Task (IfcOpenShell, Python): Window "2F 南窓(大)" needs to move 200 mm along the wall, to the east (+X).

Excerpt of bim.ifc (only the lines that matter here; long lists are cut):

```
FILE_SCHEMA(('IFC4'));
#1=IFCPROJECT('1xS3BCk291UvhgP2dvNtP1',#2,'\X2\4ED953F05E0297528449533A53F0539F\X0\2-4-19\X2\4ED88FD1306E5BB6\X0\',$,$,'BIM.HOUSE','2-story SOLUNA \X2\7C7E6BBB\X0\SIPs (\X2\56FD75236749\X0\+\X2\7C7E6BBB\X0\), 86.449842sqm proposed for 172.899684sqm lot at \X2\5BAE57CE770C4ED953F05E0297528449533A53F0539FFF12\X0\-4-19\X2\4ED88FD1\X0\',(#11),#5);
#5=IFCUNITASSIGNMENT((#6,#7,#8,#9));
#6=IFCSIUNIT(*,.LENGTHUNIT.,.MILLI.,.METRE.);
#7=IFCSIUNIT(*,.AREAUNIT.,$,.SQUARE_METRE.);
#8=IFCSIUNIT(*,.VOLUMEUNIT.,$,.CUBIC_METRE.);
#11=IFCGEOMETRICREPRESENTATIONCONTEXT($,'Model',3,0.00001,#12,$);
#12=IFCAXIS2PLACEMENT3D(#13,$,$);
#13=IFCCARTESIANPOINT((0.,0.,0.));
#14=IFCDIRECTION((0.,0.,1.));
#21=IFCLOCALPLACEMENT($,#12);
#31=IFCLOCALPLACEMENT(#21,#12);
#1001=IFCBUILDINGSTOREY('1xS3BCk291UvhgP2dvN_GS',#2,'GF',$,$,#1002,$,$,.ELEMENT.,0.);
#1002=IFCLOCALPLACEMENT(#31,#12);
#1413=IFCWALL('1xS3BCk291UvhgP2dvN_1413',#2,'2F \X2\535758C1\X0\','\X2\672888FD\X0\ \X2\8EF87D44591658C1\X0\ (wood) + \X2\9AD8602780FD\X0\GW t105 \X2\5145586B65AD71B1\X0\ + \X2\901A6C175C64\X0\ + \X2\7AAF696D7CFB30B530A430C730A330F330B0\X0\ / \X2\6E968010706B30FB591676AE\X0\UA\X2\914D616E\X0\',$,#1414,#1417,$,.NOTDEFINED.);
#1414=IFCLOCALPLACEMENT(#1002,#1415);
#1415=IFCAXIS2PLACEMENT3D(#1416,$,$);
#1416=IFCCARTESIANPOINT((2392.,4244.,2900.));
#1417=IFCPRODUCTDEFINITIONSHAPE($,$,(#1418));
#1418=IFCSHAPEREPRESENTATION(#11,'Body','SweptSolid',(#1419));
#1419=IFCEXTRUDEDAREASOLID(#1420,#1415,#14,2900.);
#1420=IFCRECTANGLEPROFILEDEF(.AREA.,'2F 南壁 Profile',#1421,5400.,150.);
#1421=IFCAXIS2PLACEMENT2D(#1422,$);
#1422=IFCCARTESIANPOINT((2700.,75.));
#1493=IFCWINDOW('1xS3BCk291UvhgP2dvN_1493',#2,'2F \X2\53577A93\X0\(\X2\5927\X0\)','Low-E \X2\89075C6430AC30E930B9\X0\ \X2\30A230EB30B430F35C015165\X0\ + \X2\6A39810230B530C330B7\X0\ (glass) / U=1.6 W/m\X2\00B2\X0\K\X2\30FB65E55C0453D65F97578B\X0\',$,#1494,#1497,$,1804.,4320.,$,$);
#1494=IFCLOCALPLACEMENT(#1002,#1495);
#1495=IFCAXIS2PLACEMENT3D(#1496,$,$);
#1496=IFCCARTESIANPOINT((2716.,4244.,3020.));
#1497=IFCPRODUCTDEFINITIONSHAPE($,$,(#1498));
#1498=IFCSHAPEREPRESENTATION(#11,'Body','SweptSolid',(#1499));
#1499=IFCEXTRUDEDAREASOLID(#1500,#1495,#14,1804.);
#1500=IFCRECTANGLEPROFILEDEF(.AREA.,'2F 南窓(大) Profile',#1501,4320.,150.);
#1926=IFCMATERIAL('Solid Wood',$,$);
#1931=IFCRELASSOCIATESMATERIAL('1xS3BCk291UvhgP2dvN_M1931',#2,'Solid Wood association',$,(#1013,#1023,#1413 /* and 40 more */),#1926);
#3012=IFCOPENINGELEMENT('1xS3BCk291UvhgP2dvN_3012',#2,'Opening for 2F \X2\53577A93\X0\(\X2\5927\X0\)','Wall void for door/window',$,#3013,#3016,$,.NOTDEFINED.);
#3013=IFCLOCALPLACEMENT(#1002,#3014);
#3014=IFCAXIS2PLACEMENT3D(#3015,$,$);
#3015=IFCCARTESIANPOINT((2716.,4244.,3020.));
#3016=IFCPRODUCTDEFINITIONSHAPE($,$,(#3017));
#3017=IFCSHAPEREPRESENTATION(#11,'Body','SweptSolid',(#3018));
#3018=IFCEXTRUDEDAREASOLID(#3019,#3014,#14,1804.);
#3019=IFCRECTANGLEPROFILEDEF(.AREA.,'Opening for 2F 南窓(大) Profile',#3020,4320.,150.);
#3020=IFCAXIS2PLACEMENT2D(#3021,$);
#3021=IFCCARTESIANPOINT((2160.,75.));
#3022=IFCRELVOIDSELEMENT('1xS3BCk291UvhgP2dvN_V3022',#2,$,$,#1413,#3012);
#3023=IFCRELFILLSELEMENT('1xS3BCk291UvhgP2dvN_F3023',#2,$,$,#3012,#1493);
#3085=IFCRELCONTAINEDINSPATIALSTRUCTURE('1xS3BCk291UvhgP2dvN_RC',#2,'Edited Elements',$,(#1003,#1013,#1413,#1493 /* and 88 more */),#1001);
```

```python
import ifcopenshell
import ifcopenshell.api.geometry
import ifcopenshell.util.placement

model = ifcopenshell.open("bim.ifc")

window = model.by_id(1493)
opening = window.FillsVoids[0].RelatingOpeningElement
wall = opening.VoidsElements[0].RelatingBuildingElement

wall_matrix = ifcopenshell.util.placement.get_local_placement(wall.ObjectPlacement)
shift = wall_matrix[:3, 0] * 200.0
before = ifcopenshell.util.placement.get_local_placement(window.ObjectPlacement)[:3, 3].copy()

# The window is not placed relative to its opening, so move both.
for product in (opening, window):
    matrix = ifcopenshell.util.placement.get_local_placement(product.ObjectPlacement)
    matrix[:3, 3] += shift
    ifcopenshell.api.geometry.edit_object_placement(model, product=product, matrix=matrix, is_si=False)

after = ifcopenshell.util.placement.get_local_placement(window.ObjectPlacement)[:3, 3]
print("window moved by", (after - before).round(3) + 0.0)

model.write("bim_rev.ifc")
```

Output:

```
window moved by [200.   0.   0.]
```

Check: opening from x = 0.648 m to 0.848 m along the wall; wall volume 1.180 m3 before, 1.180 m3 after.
